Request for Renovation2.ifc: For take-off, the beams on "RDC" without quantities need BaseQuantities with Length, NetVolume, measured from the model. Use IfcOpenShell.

First a look at what the model holds.

```python
import ifcopenshell
import ifcopenshell.util.element
import ifcopenshell.util.unit

model = ifcopenshell.open("Renovation2.ifc")
print(model.schema)
for unit_type in ("LENGTHUNIT", "AREAUNIT", "VOLUMEUNIT"):
    print(unit_type, ifcopenshell.util.unit.calculate_unit_scale(model, unit_type))
storey = next(s for s in model.by_type("IfcBuildingStorey") if s.Name == "RDC")
beams = [e for e in ifcopenshell.util.element.get_decomposition(storey) if e.is_a("IfcBeam")]
for e in sorted(beams, key=lambda e: e.id()):
    print(e.id(), e.is_a(), e.Name, list(ifcopenshell.util.element.get_psets(e, qtos_only=True)), sep=" | ")
```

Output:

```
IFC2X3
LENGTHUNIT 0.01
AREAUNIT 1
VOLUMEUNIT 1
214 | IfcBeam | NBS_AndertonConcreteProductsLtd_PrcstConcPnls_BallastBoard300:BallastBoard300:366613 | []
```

```python
import ifcopenshell
import ifcopenshell.api.pset
import ifcopenshell.geom
import ifcopenshell.util.element
import ifcopenshell.util.shape
import ifcopenshell.util.unit

model = ifcopenshell.open("Renovation2.ifc")
unit_scale = ifcopenshell.util.unit.calculate_unit_scale(model)
volume_scale = ifcopenshell.util.unit.calculate_unit_scale(model, "VOLUMEUNIT")
settings = ifcopenshell.geom.settings()

storey = next(s for s in model.by_type("IfcBuildingStorey") if s.Name == "RDC")
beams = [e for e in ifcopenshell.util.element.get_decomposition(storey) if e.is_a("IfcBeam")]

for e in sorted(beams, key=lambda e: e.id()):
    if ifcopenshell.util.element.get_psets(e, qtos_only=True, should_inherit=False):
        continue
    # Geometry comes back in metres, in the element's own axes.
    shape = ifcopenshell.geom.create_shape(settings, e)
    values = {
        "Length": ifcopenshell.util.shape.get_max_xyz(shape.geometry) / unit_scale,
        "NetVolume": ifcopenshell.util.shape.get_volume(shape.geometry) / volume_scale,
    }
    qto = ifcopenshell.api.pset.add_qto(model, product=e, name="BaseQuantities")
    ifcopenshell.api.pset.edit_qto(model, qto=qto, properties=values)
    print(e.id(), {k: round(v, 3) for k, v in values.items()})

model.write("Renovation2_updated.ifc")
```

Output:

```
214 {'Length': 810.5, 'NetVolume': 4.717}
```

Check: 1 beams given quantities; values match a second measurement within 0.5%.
